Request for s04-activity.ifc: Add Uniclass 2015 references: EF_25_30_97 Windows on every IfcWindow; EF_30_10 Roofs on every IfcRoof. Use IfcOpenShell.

First a look at what the model holds.

```python
import ifcopenshell

model = ifcopenshell.open("s04-activity.ifc")
print(model.schema)
print("classifications:", [c.Name for c in model.by_type("IfcClassification")])
for ifc_class in ("IfcDoor", "IfcRoof", "IfcStair", "IfcWall", "IfcWindow"):
    print(ifc_class, len(model.by_type(ifc_class)))
```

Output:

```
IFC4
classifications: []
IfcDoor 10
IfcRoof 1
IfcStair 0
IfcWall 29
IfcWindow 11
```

```python
import ifcopenshell
import ifcopenshell.api.classification

model = ifcopenshell.open("s04-activity.ifc")

system = ifcopenshell.api.classification.add_classification(model, classification="Uniclass 2015")

codes = {
    "IfcWindow": ("EF_25_30_97", "Windows"),
    "IfcRoof": ("EF_30_10", "Roofs"),
}
for ifc_class, (code, name) in codes.items():
    products = model.by_type(ifc_class)
    ifcopenshell.api.classification.add_reference(
        model, products=products, classification=system, identification=code, name=name
    )
    print(code, len(products))

model.write("s04-activity_rev.ifc")
```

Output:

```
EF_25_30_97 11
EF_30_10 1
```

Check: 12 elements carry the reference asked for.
